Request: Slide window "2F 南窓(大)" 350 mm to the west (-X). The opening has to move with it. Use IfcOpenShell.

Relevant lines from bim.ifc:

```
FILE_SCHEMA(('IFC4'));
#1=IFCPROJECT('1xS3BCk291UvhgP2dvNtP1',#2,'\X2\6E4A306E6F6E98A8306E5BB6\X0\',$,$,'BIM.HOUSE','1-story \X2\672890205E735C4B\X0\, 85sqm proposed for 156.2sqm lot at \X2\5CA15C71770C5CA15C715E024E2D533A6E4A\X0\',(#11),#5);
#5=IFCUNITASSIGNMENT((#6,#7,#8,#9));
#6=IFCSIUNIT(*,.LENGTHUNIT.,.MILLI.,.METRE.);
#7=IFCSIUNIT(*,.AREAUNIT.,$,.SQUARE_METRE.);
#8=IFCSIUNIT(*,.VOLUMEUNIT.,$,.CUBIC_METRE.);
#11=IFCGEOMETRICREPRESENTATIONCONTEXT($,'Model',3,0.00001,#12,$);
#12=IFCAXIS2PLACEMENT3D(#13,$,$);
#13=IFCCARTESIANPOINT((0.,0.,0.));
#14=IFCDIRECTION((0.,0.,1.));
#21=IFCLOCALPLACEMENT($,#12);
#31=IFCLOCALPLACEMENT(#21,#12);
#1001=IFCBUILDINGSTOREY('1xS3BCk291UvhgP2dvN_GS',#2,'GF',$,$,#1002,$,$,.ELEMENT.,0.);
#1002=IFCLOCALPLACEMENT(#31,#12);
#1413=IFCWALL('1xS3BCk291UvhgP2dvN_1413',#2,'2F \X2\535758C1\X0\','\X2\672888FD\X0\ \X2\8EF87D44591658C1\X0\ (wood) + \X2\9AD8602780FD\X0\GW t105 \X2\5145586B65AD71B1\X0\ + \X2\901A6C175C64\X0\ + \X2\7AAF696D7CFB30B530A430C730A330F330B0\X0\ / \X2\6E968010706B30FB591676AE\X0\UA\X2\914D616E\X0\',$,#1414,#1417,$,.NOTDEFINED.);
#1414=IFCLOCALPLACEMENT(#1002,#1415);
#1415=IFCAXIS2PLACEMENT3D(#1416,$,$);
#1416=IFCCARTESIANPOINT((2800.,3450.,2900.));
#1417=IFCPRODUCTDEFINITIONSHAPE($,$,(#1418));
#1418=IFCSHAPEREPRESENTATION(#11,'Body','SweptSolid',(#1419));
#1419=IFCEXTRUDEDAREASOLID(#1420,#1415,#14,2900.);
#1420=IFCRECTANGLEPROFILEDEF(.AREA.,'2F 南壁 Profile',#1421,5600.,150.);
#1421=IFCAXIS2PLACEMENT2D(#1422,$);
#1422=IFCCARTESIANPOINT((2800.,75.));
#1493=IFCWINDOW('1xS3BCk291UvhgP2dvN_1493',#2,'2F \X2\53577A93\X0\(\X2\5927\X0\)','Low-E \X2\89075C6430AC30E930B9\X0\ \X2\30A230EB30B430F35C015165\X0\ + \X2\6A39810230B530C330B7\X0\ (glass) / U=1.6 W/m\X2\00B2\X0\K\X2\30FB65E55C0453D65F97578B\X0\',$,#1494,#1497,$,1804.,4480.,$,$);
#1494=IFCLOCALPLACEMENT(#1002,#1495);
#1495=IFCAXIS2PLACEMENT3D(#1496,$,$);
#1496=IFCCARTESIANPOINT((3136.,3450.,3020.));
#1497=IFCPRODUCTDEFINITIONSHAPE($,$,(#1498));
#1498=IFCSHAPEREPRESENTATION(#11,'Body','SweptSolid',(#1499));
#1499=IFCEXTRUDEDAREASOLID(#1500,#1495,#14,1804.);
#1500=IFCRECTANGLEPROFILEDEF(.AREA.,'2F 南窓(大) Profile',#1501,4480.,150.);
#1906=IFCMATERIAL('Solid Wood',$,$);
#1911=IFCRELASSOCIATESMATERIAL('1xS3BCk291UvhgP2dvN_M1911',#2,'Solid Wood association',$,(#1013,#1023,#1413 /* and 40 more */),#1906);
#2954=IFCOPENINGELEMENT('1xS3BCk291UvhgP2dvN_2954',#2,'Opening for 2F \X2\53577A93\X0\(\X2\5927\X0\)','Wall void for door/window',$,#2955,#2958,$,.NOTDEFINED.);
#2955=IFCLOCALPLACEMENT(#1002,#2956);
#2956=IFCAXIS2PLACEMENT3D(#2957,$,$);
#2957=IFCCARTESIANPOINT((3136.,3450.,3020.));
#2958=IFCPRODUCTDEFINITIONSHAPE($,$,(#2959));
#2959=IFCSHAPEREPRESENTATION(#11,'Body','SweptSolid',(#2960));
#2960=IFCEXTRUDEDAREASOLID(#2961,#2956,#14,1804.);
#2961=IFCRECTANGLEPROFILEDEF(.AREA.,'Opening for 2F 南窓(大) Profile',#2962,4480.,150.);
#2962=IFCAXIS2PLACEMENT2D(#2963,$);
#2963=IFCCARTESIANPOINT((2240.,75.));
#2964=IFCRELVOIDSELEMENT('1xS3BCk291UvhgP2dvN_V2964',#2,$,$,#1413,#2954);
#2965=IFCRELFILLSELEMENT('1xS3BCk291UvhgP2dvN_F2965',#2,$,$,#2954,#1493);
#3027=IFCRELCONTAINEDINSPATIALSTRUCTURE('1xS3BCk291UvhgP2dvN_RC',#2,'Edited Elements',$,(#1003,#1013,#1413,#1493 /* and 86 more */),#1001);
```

```python
import ifcopenshell
import ifcopenshell.api.geometry
import ifcopenshell.util.placement
import ifcopenshell.util.unit

model = ifcopenshell.open("bim.ifc")
unit_scale = ifcopenshell.util.unit.calculate_unit_scale(model)

window = model.by_guid("1xS3BCk291UvhgP2dvN_1493")
opening = window.FillsVoids[0].RelatingOpeningElement
wall = opening.VoidsElements[0].RelatingBuildingElement

wall_matrix = ifcopenshell.util.placement.get_local_placement(wall.ObjectPlacement)
shift = wall_matrix[:3, 0] * -0.35 / unit_scale
before = ifcopenshell.util.placement.get_local_placement(window.ObjectPlacement)[:3, 3].copy()

# The window is not placed relative to its opening, so move both.
for product in (opening, window):
    matrix = ifcopenshell.util.placement.get_local_placement(product.ObjectPlacement)
    matrix[:3, 3] += shift
    ifcopenshell.api.geometry.edit_object_placement(model, product=product, matrix=matrix, is_si=False)

after = ifcopenshell.util.placement.get_local_placement(window.ObjectPlacement)[:3, 3]
print("window moved by", (after - before).round(3) + 0.0)

model.write("bim_rev.ifc")
```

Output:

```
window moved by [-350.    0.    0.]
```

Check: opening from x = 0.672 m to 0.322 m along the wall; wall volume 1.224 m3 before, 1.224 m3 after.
